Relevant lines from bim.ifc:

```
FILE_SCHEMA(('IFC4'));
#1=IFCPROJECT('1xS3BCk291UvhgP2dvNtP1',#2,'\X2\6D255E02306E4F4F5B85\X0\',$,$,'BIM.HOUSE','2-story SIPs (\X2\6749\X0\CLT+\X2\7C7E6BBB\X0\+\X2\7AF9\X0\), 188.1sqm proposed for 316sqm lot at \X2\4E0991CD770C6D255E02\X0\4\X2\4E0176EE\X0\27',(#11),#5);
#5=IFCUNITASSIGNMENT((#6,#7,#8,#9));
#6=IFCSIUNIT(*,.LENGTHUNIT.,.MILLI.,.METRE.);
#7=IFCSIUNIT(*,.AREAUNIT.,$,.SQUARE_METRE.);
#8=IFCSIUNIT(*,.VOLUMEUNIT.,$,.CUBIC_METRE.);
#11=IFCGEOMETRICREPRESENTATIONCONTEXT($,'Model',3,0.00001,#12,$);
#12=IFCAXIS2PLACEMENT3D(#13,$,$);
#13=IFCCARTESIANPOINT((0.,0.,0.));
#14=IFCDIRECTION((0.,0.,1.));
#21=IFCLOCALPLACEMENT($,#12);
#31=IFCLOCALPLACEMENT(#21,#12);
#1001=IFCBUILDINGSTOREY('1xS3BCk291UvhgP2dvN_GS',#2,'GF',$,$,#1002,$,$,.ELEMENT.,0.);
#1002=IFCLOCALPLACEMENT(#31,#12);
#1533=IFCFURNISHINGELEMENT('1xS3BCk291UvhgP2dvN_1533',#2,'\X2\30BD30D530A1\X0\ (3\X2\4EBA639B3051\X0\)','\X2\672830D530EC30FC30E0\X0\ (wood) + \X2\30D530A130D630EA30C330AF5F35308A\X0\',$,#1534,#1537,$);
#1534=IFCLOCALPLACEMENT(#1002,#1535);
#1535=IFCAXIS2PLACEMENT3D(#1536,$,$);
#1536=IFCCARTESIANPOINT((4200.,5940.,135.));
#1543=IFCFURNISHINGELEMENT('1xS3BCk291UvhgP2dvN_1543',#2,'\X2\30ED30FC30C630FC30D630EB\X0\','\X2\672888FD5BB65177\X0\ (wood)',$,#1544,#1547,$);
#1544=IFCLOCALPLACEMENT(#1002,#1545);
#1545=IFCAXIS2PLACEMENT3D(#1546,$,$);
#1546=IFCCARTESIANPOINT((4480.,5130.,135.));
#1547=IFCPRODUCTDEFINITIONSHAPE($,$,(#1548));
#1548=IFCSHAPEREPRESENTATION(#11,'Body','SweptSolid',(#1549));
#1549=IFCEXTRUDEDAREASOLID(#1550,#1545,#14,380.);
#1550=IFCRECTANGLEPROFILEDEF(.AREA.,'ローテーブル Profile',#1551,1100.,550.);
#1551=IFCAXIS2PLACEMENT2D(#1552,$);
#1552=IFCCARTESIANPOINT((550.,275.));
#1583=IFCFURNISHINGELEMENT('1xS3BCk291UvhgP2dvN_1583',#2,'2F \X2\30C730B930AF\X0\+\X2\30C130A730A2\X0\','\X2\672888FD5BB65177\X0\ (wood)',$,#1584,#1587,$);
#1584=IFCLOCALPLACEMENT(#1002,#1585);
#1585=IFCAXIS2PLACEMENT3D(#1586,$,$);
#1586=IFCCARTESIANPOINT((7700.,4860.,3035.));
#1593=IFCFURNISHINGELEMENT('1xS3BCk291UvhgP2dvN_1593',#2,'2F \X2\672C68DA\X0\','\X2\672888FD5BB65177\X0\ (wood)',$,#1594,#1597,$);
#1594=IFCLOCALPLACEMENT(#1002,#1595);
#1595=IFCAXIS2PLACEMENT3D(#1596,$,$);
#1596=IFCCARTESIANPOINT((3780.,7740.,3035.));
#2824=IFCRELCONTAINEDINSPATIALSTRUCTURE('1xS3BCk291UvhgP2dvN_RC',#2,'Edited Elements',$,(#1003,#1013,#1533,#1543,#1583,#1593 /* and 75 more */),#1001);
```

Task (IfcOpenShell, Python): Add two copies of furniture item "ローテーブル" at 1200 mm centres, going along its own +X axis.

```python
import ifcopenshell
import ifcopenshell.api.geometry
import ifcopenshell.api.root
import ifcopenshell.util.element
import ifcopenshell.util.placement

model = ifcopenshell.open("bim.ifc")


def reuse_history(source, copy):
    """copy_class also copies each property set's owner history, people and application; keep the originals."""
    for rel in copy.IsDefinedBy:
        if rel.is_a("IfcRelDefinesByProperties") and (history := rel.RelatingPropertyDefinition.OwnerHistory):
            rel.RelatingPropertyDefinition.OwnerHistory = source.OwnerHistory
            ifcopenshell.util.element.remove_deep2(model, history)


source = model.by_guid("1xS3BCk291UvhgP2dvN_1543")
base = ifcopenshell.util.placement.get_local_placement(source.ObjectPlacement)
step = base[:3, 0] * 1200.0

for i in range(1, 3):
    copy = ifcopenshell.api.root.copy_class(model, product=source)
    copy.Representation = ifcopenshell.util.element.copy_deep(
        model, source.Representation, exclude=["IfcGeometricRepresentationContext", "IfcRepresentationMap"]
    )
    reuse_history(source, copy)
    matrix = base.copy()
    matrix[:3, 3] += i * step
    print("added at", matrix[:3, 3].round(3) + 0.0)
    ifcopenshell.api.geometry.edit_object_placement(model, product=copy, matrix=matrix, is_si=False)

model.write("bim_edited.ifc")
```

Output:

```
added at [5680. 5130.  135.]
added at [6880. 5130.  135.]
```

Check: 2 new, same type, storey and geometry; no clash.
